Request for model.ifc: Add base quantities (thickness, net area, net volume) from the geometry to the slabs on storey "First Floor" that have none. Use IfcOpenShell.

First a look at what the model holds.

```python
import ifcopenshell
import ifcopenshell.util.element
import ifcopenshell.util.unit

model = ifcopenshell.open("model.ifc")
print(model.schema)
for unit_type in ("LENGTHUNIT", "AREAUNIT", "VOLUMEUNIT"):
    print(unit_type, ifcopenshell.util.unit.calculate_unit_scale(model, unit_type))
storey = next(s for s in model.by_type("IfcBuildingStorey") if s.Name == "First Floor")
slabs = [e for e in ifcopenshell.util.element.get_decomposition(storey) if e.is_a("IfcSlab")]
for e in sorted(slabs, key=lambda e: e.id()):
    print(e.id(), e.is_a(), e.Name, list(ifcopenshell.util.element.get_psets(e, qtos_only=True)), sep=" | ")
```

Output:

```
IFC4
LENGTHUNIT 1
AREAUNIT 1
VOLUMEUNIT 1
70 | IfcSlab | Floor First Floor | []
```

```python
import ifcopenshell
import ifcopenshell.api.pset
import ifcopenshell.geom
import ifcopenshell.util.element
import ifcopenshell.util.shape
import ifcopenshell.util.unit

model = ifcopenshell.open("model.ifc")
unit_scale = ifcopenshell.util.unit.calculate_unit_scale(model)
area_scale = ifcopenshell.util.unit.calculate_unit_scale(model, "AREAUNIT")
volume_scale = ifcopenshell.util.unit.calculate_unit_scale(model, "VOLUMEUNIT")
settings = ifcopenshell.geom.settings()

storey = next(s for s in model.by_type("IfcBuildingStorey") if s.Name == "First Floor")
slabs = [e for e in ifcopenshell.util.element.get_decomposition(storey) if e.is_a("IfcSlab")]

for e in sorted(slabs, key=lambda e: e.id()):
    if ifcopenshell.util.element.get_psets(e, qtos_only=True, should_inherit=False):
        continue
    # Geometry comes back in metres, in the element's own axes.
    shape = ifcopenshell.geom.create_shape(settings, e)
    values = {
        "Width": ifcopenshell.util.shape.get_z(shape.geometry) / unit_scale,
        "NetArea": ifcopenshell.util.shape.get_footprint_area(shape.geometry) / area_scale,
        "NetVolume": ifcopenshell.util.shape.get_volume(shape.geometry) / volume_scale,
    }
    qto = ifcopenshell.api.pset.add_qto(model, product=e, name="Qto_SlabBaseQuantities")
    ifcopenshell.api.pset.edit_qto(model, qto=qto, properties=values)
    print(e.id(), {k: round(v, 3) for k, v in values.items()})

model.write("model_rev.ifc")
```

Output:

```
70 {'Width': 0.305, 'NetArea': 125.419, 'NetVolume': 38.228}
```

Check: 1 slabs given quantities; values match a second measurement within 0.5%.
